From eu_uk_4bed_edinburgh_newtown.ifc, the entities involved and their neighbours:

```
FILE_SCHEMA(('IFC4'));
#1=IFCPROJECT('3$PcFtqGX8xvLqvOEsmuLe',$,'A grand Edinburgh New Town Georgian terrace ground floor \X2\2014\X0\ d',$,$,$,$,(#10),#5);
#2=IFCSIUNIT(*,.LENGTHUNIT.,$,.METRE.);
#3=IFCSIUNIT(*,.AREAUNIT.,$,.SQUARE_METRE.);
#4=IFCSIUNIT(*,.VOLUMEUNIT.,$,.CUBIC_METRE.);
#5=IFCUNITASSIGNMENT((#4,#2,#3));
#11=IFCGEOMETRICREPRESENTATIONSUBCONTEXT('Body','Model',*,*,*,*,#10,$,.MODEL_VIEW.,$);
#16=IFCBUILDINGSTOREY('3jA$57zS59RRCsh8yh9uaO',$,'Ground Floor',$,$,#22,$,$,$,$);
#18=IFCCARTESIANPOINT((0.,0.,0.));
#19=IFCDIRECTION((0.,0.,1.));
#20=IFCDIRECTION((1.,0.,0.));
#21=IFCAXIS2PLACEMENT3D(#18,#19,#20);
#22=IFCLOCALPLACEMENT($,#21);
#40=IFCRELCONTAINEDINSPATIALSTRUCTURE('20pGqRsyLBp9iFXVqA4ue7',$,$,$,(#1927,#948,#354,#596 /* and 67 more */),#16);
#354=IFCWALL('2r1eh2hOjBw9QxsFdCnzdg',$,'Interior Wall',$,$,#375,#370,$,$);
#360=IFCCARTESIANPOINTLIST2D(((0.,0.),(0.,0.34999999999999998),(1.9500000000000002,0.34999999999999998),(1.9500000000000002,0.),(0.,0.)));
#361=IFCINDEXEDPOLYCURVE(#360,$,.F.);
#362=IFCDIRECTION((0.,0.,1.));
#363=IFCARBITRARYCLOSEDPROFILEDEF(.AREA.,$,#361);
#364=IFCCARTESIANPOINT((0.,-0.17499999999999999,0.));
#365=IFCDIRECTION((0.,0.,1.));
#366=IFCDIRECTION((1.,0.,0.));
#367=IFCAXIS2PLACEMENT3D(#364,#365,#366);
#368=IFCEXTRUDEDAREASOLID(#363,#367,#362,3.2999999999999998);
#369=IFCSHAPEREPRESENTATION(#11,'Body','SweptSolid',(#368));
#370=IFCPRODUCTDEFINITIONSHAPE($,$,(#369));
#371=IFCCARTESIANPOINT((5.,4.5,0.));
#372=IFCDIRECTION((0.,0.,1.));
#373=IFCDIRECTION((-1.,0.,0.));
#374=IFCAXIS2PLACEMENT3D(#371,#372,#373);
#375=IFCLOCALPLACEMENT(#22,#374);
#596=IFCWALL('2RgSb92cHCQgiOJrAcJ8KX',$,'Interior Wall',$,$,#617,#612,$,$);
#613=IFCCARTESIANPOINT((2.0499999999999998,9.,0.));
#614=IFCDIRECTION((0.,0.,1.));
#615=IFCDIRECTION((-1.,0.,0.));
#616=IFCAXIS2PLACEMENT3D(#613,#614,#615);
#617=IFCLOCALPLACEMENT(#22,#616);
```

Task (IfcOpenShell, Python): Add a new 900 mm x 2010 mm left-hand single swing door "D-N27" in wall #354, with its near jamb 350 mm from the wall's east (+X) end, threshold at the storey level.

```python
import numpy as np
import ifcopenshell
import ifcopenshell.api.feature
import ifcopenshell.api.geometry
import ifcopenshell.api.root
import ifcopenshell.api.spatial
import ifcopenshell.geom
import ifcopenshell.util.element
import ifcopenshell.util.placement
import ifcopenshell.util.representation
import ifcopenshell.util.shape
import ifcopenshell.util.unit

model = ifcopenshell.open("eu_uk_4bed_edinburgh_newtown.ifc")
unit_scale = ifcopenshell.util.unit.calculate_unit_scale(model)
settings = ifcopenshell.geom.settings()


def volume(element):
    """Net volume in cubic metres, openings subtracted."""
    shape = ifcopenshell.geom.create_shape(settings, element)
    return ifcopenshell.util.shape.get_volume(shape.geometry)


wall = model.by_guid("2r1eh2hOjBw9QxsFdCnzdg")
storey = ifcopenshell.util.element.get_container(wall, ifc_class="IfcBuildingStorey")
context = ifcopenshell.util.representation.get_context(model, "Model", "Body", "MODEL_VIEW")
before = volume(wall)

width, height, from_end, sill = 0.9, 2.01, 0.35, 0.0  # metres

# The wall runs along its own X axis, and the end named is its -X end.
wall_shape = ifcopenshell.geom.create_shape(settings, wall)
x, y, z = ifcopenshell.util.shape.get_vertices(wall_shape.geometry).T
start = x.min() + from_end
face, thickness = float(y.min()), float(y.max() - y.min())
wall_matrix = ifcopenshell.util.placement.get_local_placement(wall.ObjectPlacement)
level = ifcopenshell.util.placement.get_local_placement(storey.ObjectPlacement)[2, 3]


def in_wall(x, y):
    """Placement at x, y metres in the wall's axes, at sill height."""
    matrix = wall_matrix.copy()
    matrix[:, 3] = wall_matrix @ np.array([x / unit_scale, y / unit_scale, 0.0, 1.0])
    matrix[2, 3] = level + sill / unit_scale
    return matrix


# Opening: a box that overshoots both wall faces by 50 mm.
opening = ifcopenshell.api.root.create_entity(model, ifc_class="IfcOpeningElement", predefined_type="OPENING")
box = ifcopenshell.api.geometry.add_wall_representation(
    model, context=context, length=width, height=height, thickness=thickness + 0.1
)
ifcopenshell.api.geometry.assign_representation(model, product=opening, representation=box)
ifcopenshell.api.geometry.edit_object_placement(model, product=opening, matrix=in_wall(start, face - 0.05), is_si=False)
ifcopenshell.api.feature.add_feature(model, feature=opening, element=wall)

door = ifcopenshell.api.root.create_entity(model, ifc_class="IfcDoor", name="D-N27", predefined_type="DOOR")
door.OverallWidth, door.OverallHeight = width / unit_scale, height / unit_scale
door.OperationType = "SINGLE_SWING_LEFT"
body = ifcopenshell.api.geometry.add_door_representation(
    model,
    context=context,
    overall_width=door.OverallWidth,
    overall_height=door.OverallHeight,
    operation_type="SINGLE_SWING_LEFT",
    lining_properties={"LiningDepth": thickness / unit_scale, "ThresholdDepth": thickness / unit_scale},
)
ifcopenshell.api.geometry.assign_representation(model, product=door, representation=body)
ifcopenshell.api.spatial.assign_container(model, products=[door], relating_structure=storey)
ifcopenshell.api.feature.add_filling(model, opening=opening, element=door)

# The lining spans the wall, so the door starts at the wall face.
ifcopenshell.api.geometry.edit_object_placement(model, product=door, matrix=in_wall(start, face), is_si=False)

after = volume(wall)

print(f"wall volume {before:.3f} -> {after:.3f} m3")

model.write("eu_uk_4bed_edinburgh_newtown_edited.ifc")
```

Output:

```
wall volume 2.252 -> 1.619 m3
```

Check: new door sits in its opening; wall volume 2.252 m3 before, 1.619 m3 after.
